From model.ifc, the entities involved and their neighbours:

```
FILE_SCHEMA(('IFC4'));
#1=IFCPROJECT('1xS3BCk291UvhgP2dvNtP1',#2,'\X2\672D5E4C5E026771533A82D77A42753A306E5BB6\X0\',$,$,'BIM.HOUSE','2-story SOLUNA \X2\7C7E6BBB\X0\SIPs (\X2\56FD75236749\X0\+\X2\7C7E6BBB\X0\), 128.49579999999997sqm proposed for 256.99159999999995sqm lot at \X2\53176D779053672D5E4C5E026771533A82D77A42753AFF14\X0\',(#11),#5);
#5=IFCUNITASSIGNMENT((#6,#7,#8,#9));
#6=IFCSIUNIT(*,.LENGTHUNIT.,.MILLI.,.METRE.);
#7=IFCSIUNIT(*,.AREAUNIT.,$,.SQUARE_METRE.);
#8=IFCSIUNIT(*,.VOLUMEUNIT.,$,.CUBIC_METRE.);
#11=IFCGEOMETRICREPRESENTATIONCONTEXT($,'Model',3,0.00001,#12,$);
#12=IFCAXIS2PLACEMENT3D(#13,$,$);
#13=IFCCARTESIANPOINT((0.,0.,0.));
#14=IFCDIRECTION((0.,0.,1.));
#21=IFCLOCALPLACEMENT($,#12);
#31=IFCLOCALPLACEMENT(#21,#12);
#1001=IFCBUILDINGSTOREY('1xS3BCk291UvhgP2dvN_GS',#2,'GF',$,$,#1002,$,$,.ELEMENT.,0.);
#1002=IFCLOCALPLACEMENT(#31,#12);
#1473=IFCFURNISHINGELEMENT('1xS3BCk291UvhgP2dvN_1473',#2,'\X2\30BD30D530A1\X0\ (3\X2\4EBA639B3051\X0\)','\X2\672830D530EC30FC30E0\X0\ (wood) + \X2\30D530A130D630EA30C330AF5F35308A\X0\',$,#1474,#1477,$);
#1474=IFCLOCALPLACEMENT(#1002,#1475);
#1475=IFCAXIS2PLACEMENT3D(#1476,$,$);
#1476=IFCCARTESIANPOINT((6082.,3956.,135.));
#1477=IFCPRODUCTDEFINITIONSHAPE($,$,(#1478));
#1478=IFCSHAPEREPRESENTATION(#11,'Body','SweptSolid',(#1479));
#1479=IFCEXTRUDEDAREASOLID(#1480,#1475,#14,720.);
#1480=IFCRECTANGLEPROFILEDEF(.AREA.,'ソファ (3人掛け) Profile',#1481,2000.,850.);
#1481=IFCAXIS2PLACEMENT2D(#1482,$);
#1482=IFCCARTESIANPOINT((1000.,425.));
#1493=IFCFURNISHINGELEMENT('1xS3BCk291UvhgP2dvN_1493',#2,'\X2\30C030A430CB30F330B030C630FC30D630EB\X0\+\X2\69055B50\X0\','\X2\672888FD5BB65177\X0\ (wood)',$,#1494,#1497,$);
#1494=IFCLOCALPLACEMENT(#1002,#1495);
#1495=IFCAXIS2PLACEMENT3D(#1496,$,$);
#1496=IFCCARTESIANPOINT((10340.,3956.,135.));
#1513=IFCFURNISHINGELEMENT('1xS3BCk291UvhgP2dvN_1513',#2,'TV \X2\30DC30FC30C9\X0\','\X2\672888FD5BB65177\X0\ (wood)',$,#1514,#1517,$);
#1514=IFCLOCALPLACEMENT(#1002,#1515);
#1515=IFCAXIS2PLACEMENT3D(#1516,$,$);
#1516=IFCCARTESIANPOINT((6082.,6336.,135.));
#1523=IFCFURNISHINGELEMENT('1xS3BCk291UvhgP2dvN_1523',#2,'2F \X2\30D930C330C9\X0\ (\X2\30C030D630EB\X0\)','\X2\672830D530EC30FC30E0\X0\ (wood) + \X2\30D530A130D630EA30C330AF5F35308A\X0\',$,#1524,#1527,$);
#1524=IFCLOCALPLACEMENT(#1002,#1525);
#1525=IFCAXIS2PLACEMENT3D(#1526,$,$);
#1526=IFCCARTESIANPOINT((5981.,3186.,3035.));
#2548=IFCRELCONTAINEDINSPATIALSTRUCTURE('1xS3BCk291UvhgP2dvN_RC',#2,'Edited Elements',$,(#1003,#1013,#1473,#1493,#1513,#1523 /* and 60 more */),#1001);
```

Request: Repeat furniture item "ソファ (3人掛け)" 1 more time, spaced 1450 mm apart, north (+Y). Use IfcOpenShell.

```python
import numpy as np
import ifcopenshell
import ifcopenshell.api.geometry
import ifcopenshell.api.root
import ifcopenshell.util.element
import ifcopenshell.util.placement
import ifcopenshell.util.unit

model = ifcopenshell.open("model.ifc")
unit_scale = ifcopenshell.util.unit.calculate_unit_scale(model)


def reuse_history(source, copy):
    """copy_class also copies each property set's owner history, people and application; keep the originals."""
    for rel in copy.IsDefinedBy:
        if rel.is_a("IfcRelDefinesByProperties") and (history := rel.RelatingPropertyDefinition.OwnerHistory):
            rel.RelatingPropertyDefinition.OwnerHistory = source.OwnerHistory
            ifcopenshell.util.element.remove_deep2(model, history)


source = model.by_guid("1xS3BCk291UvhgP2dvN_1473")
base = ifcopenshell.util.placement.get_local_placement(source.ObjectPlacement)
step = np.array([0.0, 1.0, 0.0]) * 1.45 / unit_scale

for i in range(1, 2):
    copy = ifcopenshell.api.root.copy_class(model, product=source)
    copy.Representation = ifcopenshell.util.element.copy_deep(
        model, source.Representation, exclude=["IfcGeometricRepresentationContext", "IfcRepresentationMap"]
    )
    reuse_history(source, copy)
    matrix = base.copy()
    matrix[:3, 3] += i * step
    print("added at", matrix[:3, 3].round(3) + 0.0)
    ifcopenshell.api.geometry.edit_object_placement(model, product=copy, matrix=matrix, is_si=False)

model.write("model_edited.ifc")
```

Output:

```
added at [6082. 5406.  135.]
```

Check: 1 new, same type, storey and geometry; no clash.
